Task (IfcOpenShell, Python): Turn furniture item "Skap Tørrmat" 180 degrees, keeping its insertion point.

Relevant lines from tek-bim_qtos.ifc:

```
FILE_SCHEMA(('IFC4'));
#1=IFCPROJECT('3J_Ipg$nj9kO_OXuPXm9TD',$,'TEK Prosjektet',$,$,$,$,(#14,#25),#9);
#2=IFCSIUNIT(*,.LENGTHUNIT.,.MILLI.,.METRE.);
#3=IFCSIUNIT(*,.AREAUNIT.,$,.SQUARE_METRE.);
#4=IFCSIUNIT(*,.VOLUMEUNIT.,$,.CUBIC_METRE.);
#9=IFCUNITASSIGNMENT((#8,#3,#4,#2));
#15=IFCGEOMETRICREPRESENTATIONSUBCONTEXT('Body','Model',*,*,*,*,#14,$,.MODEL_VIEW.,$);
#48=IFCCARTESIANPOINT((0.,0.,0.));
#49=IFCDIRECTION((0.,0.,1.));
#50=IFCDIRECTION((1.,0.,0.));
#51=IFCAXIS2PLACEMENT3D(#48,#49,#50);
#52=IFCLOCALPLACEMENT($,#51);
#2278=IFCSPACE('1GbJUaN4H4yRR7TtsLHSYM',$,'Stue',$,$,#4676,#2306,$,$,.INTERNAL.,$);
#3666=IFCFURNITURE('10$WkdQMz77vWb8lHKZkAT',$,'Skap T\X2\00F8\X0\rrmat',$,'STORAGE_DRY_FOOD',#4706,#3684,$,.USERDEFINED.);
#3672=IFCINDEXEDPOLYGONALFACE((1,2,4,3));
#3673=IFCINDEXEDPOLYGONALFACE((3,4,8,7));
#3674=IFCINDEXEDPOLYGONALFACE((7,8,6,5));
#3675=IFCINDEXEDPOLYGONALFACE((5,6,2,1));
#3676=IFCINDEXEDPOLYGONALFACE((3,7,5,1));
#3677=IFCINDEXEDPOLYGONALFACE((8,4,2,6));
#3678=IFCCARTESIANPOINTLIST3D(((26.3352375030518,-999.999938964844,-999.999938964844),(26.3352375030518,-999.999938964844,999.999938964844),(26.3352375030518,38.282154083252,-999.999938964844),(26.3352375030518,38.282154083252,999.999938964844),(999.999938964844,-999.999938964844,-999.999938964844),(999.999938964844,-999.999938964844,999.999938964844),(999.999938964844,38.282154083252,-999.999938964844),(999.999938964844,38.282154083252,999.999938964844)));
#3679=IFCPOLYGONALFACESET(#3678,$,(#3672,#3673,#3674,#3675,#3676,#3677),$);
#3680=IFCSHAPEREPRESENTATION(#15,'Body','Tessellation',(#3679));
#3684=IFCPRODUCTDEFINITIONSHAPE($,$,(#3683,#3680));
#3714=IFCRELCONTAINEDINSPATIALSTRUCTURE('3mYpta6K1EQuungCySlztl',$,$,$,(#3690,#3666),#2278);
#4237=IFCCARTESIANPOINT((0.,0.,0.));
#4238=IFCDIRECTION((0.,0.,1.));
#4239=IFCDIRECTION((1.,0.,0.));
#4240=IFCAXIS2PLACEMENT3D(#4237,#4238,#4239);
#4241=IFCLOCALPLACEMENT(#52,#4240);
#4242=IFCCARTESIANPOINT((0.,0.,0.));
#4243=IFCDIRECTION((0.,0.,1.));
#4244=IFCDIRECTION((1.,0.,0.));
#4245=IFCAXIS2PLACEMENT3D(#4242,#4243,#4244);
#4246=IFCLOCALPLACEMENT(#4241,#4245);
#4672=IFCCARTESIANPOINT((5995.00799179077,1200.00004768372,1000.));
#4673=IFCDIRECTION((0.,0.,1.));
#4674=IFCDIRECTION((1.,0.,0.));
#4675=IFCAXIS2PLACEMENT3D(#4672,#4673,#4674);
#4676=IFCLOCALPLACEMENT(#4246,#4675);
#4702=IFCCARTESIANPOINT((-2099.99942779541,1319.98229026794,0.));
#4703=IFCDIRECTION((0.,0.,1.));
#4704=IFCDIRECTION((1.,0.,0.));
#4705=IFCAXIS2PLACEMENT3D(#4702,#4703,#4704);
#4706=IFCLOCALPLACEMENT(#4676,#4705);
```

```python
import ifcopenshell
import ifcopenshell.api.geometry
import ifcopenshell.util.placement

model = ifcopenshell.open("tek-bim_qtos.ifc")

item = model.by_id(3666)
matrix = ifcopenshell.util.placement.get_local_placement(item.ObjectPlacement)
matrix = matrix @ ifcopenshell.util.placement.rotation(180, "Z")
ifcopenshell.api.geometry.edit_object_placement(model, product=item, matrix=matrix, is_si=False)

print(ifcopenshell.util.placement.get_local_placement(item.ObjectPlacement).round(3) + 0.0)

model.write("tek-bim_qtos_updated.ifc")
```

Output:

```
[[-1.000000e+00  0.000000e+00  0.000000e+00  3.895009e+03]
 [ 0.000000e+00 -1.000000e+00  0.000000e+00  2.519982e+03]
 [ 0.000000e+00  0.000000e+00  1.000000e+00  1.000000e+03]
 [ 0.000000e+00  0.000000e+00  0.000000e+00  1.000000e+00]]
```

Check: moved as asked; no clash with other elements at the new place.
